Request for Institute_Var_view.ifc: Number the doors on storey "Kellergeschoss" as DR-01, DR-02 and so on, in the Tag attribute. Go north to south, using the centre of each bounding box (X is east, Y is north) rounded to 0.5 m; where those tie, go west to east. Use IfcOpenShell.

First a look at what the model holds.

```python
import ifcopenshell
import ifcopenshell.util.element
import ifcopenshell.util.placement

model = ifcopenshell.open("Institute_Var_view.ifc")
print(model.schema)
storey = next(s for s in model.by_type("IfcBuildingStorey") if s.Name == "Kellergeschoss")
doors = [e for e in ifcopenshell.util.element.get_decomposition(storey) if e.is_a("IfcDoor")]
for e in sorted(doors, key=lambda e: e.id()):
    origin = ifcopenshell.util.placement.get_local_placement(e.ObjectPlacement)[:3, 3]
    print(e.id(), e.Tag, e.Name, origin.round(2) + 0.0, sep=" | ")
```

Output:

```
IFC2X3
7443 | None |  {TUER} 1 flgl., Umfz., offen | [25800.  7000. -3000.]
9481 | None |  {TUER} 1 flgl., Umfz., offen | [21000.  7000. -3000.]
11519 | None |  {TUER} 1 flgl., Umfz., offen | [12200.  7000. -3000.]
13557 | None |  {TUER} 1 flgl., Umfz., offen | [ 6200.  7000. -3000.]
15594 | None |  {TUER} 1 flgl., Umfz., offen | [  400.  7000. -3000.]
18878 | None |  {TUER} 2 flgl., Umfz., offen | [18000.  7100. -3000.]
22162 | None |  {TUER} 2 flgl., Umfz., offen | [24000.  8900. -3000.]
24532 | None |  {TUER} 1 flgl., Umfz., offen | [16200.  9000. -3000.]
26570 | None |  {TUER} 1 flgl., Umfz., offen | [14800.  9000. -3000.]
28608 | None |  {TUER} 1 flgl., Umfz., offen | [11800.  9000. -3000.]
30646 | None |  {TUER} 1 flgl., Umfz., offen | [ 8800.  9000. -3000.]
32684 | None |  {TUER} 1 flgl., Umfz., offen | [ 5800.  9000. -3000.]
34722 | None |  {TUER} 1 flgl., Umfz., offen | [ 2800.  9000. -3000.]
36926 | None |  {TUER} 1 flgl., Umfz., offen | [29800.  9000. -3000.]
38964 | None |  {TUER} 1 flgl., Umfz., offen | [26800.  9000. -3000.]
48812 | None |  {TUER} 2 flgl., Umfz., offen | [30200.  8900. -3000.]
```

```python
import ifcopenshell
import ifcopenshell.geom
import ifcopenshell.util.element
import ifcopenshell.util.shape

model = ifcopenshell.open("Institute_Var_view.ifc")
settings = ifcopenshell.geom.settings()
settings.set("use-world-coords", True)


def centre(element):
    shape = ifcopenshell.geom.create_shape(settings, element)
    return ifcopenshell.util.shape.get_bbox_centroid(shape.geometry)


storey = next(s for s in model.by_type("IfcBuildingStorey") if s.Name == "Kellergeschoss")
doors = [e for e in ifcopenshell.util.element.get_decomposition(storey) if e.is_a("IfcDoor")]

# Insertion points can sit at a corner or the storey origin, so sort by the geometry (in metres).
centres = {e: centre(e) for e in doors}
doors.sort(key=lambda e: (-round(centres[e][1] / 0.5), centres[e][0]))

for i, e in enumerate(doors, start=1):
    number = f"DR-{i:02d}"
    e.Tag = number
    print(e.id(), number)

model.write("Institute_Var_view_edited.ifc")
```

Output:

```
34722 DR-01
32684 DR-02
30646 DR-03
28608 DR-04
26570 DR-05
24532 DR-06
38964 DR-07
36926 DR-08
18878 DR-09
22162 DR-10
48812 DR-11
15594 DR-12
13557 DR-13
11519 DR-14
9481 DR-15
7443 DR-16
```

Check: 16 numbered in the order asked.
